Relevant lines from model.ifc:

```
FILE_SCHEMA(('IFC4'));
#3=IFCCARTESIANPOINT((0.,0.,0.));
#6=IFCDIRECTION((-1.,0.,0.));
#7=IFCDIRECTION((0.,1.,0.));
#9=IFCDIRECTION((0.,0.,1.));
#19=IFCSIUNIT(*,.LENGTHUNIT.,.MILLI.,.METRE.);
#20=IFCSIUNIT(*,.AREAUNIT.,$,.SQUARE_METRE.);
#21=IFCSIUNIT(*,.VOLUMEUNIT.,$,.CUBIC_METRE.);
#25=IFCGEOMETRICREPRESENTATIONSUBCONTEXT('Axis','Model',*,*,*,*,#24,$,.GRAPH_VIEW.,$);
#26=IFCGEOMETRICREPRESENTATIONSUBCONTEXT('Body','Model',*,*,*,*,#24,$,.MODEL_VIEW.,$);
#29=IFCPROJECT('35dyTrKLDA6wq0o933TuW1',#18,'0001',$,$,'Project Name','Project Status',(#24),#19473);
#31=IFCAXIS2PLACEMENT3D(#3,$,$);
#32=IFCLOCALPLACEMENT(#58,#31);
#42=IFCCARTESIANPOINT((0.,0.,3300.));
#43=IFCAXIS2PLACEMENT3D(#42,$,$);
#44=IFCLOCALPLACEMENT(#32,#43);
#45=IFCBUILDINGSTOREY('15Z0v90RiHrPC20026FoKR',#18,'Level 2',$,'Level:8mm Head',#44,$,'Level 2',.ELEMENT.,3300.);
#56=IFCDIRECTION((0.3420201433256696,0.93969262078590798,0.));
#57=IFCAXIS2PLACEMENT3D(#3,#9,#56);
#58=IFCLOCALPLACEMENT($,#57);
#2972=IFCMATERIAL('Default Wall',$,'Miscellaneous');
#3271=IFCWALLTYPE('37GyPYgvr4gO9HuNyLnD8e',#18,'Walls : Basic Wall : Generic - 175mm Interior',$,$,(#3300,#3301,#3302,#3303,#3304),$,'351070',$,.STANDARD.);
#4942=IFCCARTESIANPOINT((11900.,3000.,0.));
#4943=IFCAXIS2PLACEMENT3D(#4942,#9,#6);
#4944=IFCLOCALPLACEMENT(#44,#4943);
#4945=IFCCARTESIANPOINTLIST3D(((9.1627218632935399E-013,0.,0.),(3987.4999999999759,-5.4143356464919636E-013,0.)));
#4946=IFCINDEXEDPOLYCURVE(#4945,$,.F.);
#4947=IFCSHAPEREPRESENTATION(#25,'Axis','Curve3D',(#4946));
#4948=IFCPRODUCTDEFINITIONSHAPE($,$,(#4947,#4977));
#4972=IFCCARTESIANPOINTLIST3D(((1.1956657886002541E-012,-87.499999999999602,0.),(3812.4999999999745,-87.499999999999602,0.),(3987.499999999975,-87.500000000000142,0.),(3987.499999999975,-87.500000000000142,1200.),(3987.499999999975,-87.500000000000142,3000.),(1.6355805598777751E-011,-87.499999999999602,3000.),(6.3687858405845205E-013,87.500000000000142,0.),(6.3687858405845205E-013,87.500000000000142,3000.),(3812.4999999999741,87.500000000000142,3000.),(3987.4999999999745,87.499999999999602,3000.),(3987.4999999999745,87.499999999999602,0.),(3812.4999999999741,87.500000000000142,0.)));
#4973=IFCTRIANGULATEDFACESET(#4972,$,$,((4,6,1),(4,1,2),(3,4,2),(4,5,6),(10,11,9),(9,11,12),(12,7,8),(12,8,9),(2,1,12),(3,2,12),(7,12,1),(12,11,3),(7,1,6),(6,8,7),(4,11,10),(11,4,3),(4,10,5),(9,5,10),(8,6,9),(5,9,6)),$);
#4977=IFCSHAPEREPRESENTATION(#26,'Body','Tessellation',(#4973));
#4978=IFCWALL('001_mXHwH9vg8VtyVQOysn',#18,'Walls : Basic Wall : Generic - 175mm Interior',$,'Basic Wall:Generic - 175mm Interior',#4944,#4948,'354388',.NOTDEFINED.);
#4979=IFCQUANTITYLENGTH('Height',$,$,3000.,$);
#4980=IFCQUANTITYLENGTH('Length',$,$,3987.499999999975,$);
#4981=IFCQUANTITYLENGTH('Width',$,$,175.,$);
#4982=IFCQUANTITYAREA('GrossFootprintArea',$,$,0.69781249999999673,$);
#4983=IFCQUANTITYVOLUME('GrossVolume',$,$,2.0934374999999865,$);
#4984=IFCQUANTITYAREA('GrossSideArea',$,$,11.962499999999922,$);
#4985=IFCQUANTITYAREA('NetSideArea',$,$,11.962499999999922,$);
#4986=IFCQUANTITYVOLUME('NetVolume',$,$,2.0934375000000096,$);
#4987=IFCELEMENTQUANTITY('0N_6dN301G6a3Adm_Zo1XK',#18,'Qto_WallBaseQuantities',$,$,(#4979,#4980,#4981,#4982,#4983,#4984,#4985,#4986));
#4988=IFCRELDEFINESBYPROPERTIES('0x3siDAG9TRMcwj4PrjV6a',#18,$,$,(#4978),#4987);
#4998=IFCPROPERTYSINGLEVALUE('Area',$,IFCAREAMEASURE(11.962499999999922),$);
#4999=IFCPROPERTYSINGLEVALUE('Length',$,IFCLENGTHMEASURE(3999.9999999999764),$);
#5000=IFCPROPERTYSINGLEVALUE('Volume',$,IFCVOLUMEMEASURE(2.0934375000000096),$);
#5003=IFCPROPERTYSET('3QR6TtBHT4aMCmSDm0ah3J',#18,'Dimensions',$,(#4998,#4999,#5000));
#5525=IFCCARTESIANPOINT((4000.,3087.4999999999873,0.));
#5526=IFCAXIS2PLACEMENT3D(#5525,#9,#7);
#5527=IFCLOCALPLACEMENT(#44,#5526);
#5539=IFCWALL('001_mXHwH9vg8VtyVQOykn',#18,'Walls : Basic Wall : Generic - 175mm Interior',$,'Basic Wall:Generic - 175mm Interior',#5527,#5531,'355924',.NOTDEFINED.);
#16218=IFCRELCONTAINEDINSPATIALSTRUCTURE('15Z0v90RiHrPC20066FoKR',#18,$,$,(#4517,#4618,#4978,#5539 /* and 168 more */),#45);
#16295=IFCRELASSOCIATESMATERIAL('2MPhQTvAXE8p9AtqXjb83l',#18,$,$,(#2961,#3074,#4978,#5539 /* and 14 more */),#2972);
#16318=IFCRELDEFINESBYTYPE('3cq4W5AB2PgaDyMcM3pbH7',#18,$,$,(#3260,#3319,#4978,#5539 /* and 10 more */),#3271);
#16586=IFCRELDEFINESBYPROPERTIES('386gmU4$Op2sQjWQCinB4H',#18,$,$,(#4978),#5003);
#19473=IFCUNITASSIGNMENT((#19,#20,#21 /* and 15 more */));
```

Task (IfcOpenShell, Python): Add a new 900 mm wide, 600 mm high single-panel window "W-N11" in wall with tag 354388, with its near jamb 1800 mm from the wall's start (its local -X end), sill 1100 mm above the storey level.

```python
import numpy as np
import ifcopenshell
import ifcopenshell.api.feature
import ifcopenshell.api.geometry
import ifcopenshell.api.pset
import ifcopenshell.api.root
import ifcopenshell.api.spatial
import ifcopenshell.geom
import ifcopenshell.util.element
import ifcopenshell.util.placement
import ifcopenshell.util.representation
import ifcopenshell.util.shape
import ifcopenshell.util.unit

model = ifcopenshell.open("model.ifc")
unit_scale = ifcopenshell.util.unit.calculate_unit_scale(model)
area_scale = ifcopenshell.util.unit.calculate_unit_scale(model, "AREAUNIT")
volume_scale = ifcopenshell.util.unit.calculate_unit_scale(model, "VOLUMEUNIT")
settings = ifcopenshell.geom.settings()


def volume(element):
    """Net volume in cubic metres, openings subtracted."""
    shape = ifcopenshell.geom.create_shape(settings, element)
    return ifcopenshell.util.shape.get_volume(shape.geometry)


wall = model.by_guid("001_mXHwH9vg8VtyVQOysn")
storey = ifcopenshell.util.element.get_container(wall, ifc_class="IfcBuildingStorey")
context = ifcopenshell.util.representation.get_context(model, "Model", "Body", "MODEL_VIEW")
before = volume(wall)

width, height, from_end, sill = 0.9, 0.6, 1.8, 1.1  # metres

# The wall runs along its own X axis, and the end named is its -X end.
wall_shape = ifcopenshell.geom.create_shape(settings, wall)
x, y, z = ifcopenshell.util.shape.get_vertices(wall_shape.geometry).T
start = x.min() + from_end
face, thickness = float(y.min()), float(y.max() - y.min())
wall_matrix = ifcopenshell.util.placement.get_local_placement(wall.ObjectPlacement)
level = ifcopenshell.util.placement.get_local_placement(storey.ObjectPlacement)[2, 3]


def in_wall(x, y):
    """Placement at x, y metres in the wall's axes, at sill height."""
    matrix = wall_matrix.copy()
    matrix[:, 3] = wall_matrix @ np.array([x / unit_scale, y / unit_scale, 0.0, 1.0])
    matrix[2, 3] = level + sill / unit_scale
    return matrix


# Opening: a box that overshoots both wall faces by 50 mm.
opening = ifcopenshell.api.root.create_entity(model, ifc_class="IfcOpeningElement", predefined_type="OPENING")
box = ifcopenshell.api.geometry.add_wall_representation(
    model, context=context, length=width, height=height, thickness=thickness + 0.1
)
ifcopenshell.api.geometry.assign_representation(model, product=opening, representation=box)
ifcopenshell.api.geometry.edit_object_placement(model, product=opening, matrix=in_wall(start, face - 0.05), is_si=False)
ifcopenshell.api.feature.add_feature(model, feature=opening, element=wall)

window = ifcopenshell.api.root.create_entity(model, ifc_class="IfcWindow", name="W-N11", predefined_type="WINDOW")
window.OverallWidth, window.OverallHeight = width / unit_scale, height / unit_scale
window.PartitioningType = "SINGLE_PANEL"
body = ifcopenshell.api.geometry.add_window_representation(
    model,
    context=context,
    overall_width=window.OverallWidth,
    overall_height=window.OverallHeight,
    partition_type="SINGLE_PANEL",
)
ifcopenshell.api.geometry.assign_representation(model, product=window, representation=body)
ifcopenshell.api.spatial.assign_container(model, products=[window], relating_structure=storey)
ifcopenshell.api.feature.add_filling(model, opening=opening, element=window)

# Centre the window in the wall's thickness.
ifcopenshell.api.geometry.edit_object_placement(model, product=window, matrix=in_wall(start, face), is_si=False)
window_shape = ifcopenshell.geom.create_shape(settings, window)
depth = ifcopenshell.util.shape.get_vertices(window_shape.geometry)[:, 1]
offset = face + thickness / 2 - (depth.min() + depth.max()) / 2
ifcopenshell.api.geometry.edit_object_placement(model, product=window, matrix=in_wall(start, offset), is_si=False)

after = volume(wall)

# Update the wall's stored quantities.
qto = model.by_id(ifcopenshell.util.element.get_pset(wall, "Qto_WallBaseQuantities", should_inherit=False)["id"])
ifcopenshell.api.pset.edit_qto(model, qto=qto, properties={
    "NetSideArea": after / thickness / area_scale,
    "NetVolume": after / volume_scale,
})
pset = model.by_id(ifcopenshell.util.element.get_pset(wall, "Dimensions", should_inherit=False)["id"])
ifcopenshell.api.pset.edit_pset(model, pset=pset, properties={
    "Area": model.create_entity("IfcAreaMeasure", after / thickness / area_scale),
    "Volume": model.create_entity("IfcVolumeMeasure", after / volume_scale),
})

print(f"wall volume {before:.3f} -> {after:.3f} m3")

model.write("model-out.ifc")
```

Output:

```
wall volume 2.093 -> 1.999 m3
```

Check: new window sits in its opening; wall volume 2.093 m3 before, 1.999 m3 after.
